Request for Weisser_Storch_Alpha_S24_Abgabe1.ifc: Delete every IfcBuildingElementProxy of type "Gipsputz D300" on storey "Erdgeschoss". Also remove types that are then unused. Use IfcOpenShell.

First a look at what the model holds.

```python
import ifcopenshell
import ifcopenshell.util.element

model = ifcopenshell.open("Weisser_Storch_Alpha_S24_Abgabe1.ifc")
print(model.schema)
storey = next(s for s in model.by_type("IfcBuildingStorey") if s.Name == "Erdgeschoss")
proxies = [e for e in ifcopenshell.util.element.get_decomposition(storey) if e.is_a("IfcBuildingElementProxy")]
seen = {}
for e in proxies:
    element_type = ifcopenshell.util.element.get_type(e)
    name = element_type.Name if element_type not in (None, e) else None
    seen[name] = seen.get(name, 0) + 1
for name, count in sorted(seen.items(), key=str):
    print(count, "x", name)
```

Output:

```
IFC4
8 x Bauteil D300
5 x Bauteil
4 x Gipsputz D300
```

```python
import ifcopenshell
import ifcopenshell.api.root
import ifcopenshell.util.element

model = ifcopenshell.open("Weisser_Storch_Alpha_S24_Abgabe1.ifc")

storey = next(s for s in model.by_type("IfcBuildingStorey") if s.Name == "Erdgeschoss")
proxies = [e for e in ifcopenshell.util.element.get_decomposition(storey) if e.is_a("IfcBuildingElementProxy")]
targets = [e for e in proxies if (t := ifcopenshell.util.element.get_type(e)) not in (None, e) and t.Name == "Gipsputz D300"]
types = {ifcopenshell.util.element.get_type(e) for e in targets} - {None, *targets}

for e in targets:
    ifcopenshell.api.root.remove_product(model, product=e)
print(len(targets), "removed")

unused = [t for t in types if not ifcopenshell.util.element.get_types(t)]
for t in unused:
    ifcopenshell.api.root.remove_product(model, product=t)
print(len(unused), "unused types removed")

model.write("Weisser_Storch_Alpha_S24_Abgabe1-out.ifc")
```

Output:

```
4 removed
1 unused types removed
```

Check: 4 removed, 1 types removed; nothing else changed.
